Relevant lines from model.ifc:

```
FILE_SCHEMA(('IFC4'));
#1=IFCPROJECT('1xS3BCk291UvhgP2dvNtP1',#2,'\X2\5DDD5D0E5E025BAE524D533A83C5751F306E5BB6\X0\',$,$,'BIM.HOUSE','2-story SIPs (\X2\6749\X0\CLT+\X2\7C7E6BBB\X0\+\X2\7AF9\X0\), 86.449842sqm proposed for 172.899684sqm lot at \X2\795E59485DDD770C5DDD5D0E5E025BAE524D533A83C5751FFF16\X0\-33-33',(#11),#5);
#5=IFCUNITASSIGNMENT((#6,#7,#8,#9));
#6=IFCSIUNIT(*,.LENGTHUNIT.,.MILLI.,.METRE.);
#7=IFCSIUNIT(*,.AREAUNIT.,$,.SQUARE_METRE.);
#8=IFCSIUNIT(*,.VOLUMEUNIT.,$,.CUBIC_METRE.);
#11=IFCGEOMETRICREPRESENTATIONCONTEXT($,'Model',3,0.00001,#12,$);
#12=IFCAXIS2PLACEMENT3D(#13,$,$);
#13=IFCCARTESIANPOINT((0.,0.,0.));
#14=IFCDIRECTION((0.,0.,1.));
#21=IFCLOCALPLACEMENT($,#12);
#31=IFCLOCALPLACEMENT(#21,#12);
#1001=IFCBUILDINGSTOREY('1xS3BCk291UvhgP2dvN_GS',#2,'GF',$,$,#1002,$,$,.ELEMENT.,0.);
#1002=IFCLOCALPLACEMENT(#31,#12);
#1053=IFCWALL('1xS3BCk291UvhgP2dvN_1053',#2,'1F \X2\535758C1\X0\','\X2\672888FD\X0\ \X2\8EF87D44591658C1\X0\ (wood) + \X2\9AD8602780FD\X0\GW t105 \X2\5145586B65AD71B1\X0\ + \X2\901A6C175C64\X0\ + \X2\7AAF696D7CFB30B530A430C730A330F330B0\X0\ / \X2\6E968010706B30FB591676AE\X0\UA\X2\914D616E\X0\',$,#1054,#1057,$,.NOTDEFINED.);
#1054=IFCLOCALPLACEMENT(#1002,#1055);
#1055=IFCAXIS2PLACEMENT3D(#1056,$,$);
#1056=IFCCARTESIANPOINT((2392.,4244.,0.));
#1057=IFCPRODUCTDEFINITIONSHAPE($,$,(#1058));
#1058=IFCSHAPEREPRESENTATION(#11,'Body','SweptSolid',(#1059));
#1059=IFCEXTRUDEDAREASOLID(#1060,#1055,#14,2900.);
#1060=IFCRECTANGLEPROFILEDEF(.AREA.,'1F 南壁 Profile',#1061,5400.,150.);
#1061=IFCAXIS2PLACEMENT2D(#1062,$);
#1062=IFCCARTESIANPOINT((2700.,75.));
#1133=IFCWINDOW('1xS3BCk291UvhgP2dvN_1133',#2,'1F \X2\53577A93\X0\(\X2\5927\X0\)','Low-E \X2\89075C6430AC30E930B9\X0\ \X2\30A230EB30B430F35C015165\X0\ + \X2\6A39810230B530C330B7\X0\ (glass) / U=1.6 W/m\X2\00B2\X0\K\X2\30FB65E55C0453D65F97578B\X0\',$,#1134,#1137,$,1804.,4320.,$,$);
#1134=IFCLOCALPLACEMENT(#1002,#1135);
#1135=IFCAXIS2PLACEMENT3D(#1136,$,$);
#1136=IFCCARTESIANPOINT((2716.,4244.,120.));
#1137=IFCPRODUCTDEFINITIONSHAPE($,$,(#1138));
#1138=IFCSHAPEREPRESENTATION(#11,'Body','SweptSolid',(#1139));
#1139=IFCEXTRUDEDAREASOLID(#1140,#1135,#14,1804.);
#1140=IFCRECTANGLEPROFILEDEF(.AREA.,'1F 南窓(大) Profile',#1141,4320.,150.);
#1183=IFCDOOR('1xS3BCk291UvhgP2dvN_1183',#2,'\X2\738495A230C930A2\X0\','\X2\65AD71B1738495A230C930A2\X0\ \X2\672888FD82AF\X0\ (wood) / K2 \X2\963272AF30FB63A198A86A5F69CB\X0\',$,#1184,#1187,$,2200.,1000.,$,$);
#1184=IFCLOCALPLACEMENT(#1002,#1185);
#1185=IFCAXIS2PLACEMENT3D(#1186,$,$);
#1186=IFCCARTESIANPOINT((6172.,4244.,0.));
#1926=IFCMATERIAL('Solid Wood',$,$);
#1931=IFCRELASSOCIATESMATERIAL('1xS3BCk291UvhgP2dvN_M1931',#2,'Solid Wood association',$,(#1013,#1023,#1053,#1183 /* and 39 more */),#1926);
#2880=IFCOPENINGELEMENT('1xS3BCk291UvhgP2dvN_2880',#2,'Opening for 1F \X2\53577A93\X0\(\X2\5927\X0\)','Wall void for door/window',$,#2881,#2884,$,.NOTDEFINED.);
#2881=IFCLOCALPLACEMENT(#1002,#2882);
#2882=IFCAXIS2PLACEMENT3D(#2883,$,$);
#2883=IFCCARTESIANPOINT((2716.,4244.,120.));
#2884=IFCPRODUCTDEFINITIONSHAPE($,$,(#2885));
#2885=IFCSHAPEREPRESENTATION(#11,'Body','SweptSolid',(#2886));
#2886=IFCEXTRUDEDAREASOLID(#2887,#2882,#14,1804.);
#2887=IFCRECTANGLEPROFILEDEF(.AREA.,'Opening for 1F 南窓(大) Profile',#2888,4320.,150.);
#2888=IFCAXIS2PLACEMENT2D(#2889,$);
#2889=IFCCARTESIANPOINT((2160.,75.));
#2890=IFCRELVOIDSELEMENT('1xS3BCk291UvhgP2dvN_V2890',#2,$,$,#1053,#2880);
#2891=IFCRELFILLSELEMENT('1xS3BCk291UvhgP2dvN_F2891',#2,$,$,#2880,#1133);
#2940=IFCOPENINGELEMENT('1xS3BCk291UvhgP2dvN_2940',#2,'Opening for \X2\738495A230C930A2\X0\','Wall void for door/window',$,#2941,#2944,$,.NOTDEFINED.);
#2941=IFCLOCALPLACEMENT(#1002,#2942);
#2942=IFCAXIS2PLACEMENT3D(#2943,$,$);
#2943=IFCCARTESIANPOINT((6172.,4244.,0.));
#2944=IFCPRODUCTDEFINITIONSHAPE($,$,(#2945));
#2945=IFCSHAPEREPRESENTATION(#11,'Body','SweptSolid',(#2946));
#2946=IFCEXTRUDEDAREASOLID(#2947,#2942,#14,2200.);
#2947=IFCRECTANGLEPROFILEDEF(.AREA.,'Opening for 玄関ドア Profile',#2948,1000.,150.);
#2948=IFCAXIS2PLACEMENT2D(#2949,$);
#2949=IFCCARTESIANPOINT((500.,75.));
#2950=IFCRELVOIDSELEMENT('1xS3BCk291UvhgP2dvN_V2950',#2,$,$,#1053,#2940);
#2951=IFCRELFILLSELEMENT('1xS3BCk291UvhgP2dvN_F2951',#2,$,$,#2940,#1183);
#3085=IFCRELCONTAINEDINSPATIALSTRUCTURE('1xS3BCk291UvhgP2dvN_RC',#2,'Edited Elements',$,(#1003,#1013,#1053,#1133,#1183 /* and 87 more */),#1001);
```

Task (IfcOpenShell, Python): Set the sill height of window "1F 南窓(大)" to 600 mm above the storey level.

```python
import numpy as np
import ifcopenshell
import ifcopenshell.api.geometry
import ifcopenshell.geom
import ifcopenshell.util.element
import ifcopenshell.util.placement
import ifcopenshell.util.shape
import ifcopenshell.util.unit

model = ifcopenshell.open("model.ifc")
unit_scale = ifcopenshell.util.unit.calculate_unit_scale(model)

window = model.by_id(1133)
opening = window.FillsVoids[0].RelatingOpeningElement
storey = ifcopenshell.util.element.get_container(window, ifc_class="IfcBuildingStorey")
level = ifcopenshell.util.placement.get_local_placement(storey.ObjectPlacement)[2, 3]

# The opening's origin need not be at the sill, so measure its lowest point.
shape = ifcopenshell.geom.create_shape(ifcopenshell.geom.settings(), opening)
bottom = ifcopenshell.util.shape.get_shape_bottom_elevation(shape, shape.geometry) / unit_scale
dz = level + 0.6 / unit_scale - bottom

shift = np.array([0.0, 0.0, dz])
# The window is not placed relative to its opening, so move both.
for product in (opening, window):
    matrix = ifcopenshell.util.placement.get_local_placement(product.ObjectPlacement)
    matrix[:3, 3] += shift
    ifcopenshell.api.geometry.edit_object_placement(model, product=product, matrix=matrix, is_si=False)

print(f"moved by {dz * unit_scale:+.3f} m")

model.write("model-out.ifc")
```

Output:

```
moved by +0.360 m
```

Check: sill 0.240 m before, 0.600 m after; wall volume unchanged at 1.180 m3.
